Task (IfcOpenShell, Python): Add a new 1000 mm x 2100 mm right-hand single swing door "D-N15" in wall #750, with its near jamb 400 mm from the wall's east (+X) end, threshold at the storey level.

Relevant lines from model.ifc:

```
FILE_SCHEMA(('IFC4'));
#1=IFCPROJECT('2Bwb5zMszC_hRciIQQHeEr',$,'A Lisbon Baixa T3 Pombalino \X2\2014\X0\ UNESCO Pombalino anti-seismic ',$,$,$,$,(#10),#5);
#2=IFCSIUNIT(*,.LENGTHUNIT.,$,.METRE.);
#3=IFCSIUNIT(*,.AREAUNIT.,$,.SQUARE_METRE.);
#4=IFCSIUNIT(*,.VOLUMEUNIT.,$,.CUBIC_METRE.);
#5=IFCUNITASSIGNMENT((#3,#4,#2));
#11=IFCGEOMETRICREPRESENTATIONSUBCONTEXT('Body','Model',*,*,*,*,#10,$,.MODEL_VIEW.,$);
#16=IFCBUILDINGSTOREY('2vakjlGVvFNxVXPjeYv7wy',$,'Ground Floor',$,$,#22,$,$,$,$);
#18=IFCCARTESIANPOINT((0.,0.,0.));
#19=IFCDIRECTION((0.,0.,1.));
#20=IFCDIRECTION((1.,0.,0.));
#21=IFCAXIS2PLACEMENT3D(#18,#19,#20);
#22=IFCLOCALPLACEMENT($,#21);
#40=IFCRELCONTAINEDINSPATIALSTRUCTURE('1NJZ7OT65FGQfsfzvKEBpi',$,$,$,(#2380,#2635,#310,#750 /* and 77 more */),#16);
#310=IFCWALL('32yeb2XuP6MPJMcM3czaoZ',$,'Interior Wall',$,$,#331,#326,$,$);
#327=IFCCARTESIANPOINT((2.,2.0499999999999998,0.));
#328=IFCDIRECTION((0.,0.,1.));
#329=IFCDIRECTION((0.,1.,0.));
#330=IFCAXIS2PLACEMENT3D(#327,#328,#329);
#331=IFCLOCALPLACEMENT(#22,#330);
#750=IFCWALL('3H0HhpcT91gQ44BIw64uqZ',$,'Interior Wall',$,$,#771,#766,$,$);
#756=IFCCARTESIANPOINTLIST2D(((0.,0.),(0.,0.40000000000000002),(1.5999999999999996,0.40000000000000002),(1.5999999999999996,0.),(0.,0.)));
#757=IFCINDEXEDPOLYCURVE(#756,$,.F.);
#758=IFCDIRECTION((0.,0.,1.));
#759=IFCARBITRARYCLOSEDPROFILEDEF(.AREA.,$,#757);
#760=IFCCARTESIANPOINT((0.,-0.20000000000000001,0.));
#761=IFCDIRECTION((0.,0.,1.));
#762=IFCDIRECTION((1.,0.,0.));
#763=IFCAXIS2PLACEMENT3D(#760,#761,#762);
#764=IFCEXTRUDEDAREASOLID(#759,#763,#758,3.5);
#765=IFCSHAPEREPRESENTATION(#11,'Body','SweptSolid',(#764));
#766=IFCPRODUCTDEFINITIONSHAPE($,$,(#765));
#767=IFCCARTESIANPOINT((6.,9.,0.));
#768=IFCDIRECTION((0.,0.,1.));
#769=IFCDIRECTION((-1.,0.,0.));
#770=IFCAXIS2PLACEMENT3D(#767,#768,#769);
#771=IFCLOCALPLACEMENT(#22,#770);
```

```python
import numpy as np
import ifcopenshell
import ifcopenshell.api.feature
import ifcopenshell.api.geometry
import ifcopenshell.api.root
import ifcopenshell.api.spatial
import ifcopenshell.geom
import ifcopenshell.util.element
import ifcopenshell.util.placement
import ifcopenshell.util.representation
import ifcopenshell.util.shape
import ifcopenshell.util.unit

model = ifcopenshell.open("model.ifc")
unit_scale = ifcopenshell.util.unit.calculate_unit_scale(model)
settings = ifcopenshell.geom.settings()


def volume(element):
    """Net volume in cubic metres, openings subtracted."""
    shape = ifcopenshell.geom.create_shape(settings, element)
    return ifcopenshell.util.shape.get_volume(shape.geometry)


wall = model.by_guid("3H0HhpcT91gQ44BIw64uqZ")
storey = ifcopenshell.util.element.get_container(wall, ifc_class="IfcBuildingStorey")
context = ifcopenshell.util.representation.get_context(model, "Model", "Body", "MODEL_VIEW")
before = volume(wall)

width, height, from_end, sill = 1, 2.1, 0.4, 0.0  # metres

# The wall runs along its own X axis, and the end named is its -X end.
wall_shape = ifcopenshell.geom.create_shape(settings, wall)
x, y, z = ifcopenshell.util.shape.get_vertices(wall_shape.geometry).T
start = x.min() + from_end
face, thickness = float(y.min()), float(y.max() - y.min())
wall_matrix = ifcopenshell.util.placement.get_local_placement(wall.ObjectPlacement)
level = ifcopenshell.util.placement.get_local_placement(storey.ObjectPlacement)[2, 3]


def in_wall(x, y):
    """Placement at x, y metres in the wall's axes, at sill height."""
    matrix = wall_matrix.copy()
    matrix[:, 3] = wall_matrix @ np.array([x / unit_scale, y / unit_scale, 0.0, 1.0])
    matrix[2, 3] = level + sill / unit_scale
    return matrix


# Opening: a box that overshoots both wall faces by 50 mm.
opening = ifcopenshell.api.root.create_entity(model, ifc_class="IfcOpeningElement", predefined_type="OPENING")
box = ifcopenshell.api.geometry.add_wall_representation(
    model, context=context, length=width, height=height, thickness=thickness + 0.1
)
ifcopenshell.api.geometry.assign_representation(model, product=opening, representation=box)
ifcopenshell.api.geometry.edit_object_placement(model, product=opening, matrix=in_wall(start, face - 0.05), is_si=False)
ifcopenshell.api.feature.add_feature(model, feature=opening, element=wall)

door = ifcopenshell.api.root.create_entity(model, ifc_class="IfcDoor", name="D-N15", predefined_type="DOOR")
door.OverallWidth, door.OverallHeight = width / unit_scale, height / unit_scale
door.OperationType = "SINGLE_SWING_RIGHT"
body = ifcopenshell.api.geometry.add_door_representation(
    model,
    context=context,
    overall_width=door.OverallWidth,
    overall_height=door.OverallHeight,
    operation_type="SINGLE_SWING_RIGHT",
    lining_properties={"LiningDepth": thickness / unit_scale, "ThresholdDepth": thickness / unit_scale},
)
ifcopenshell.api.geometry.assign_representation(model, product=door, representation=body)
ifcopenshell.api.spatial.assign_container(model, products=[door], relating_structure=storey)
ifcopenshell.api.feature.add_filling(model, opening=opening, element=door)

# The lining spans the wall, so the door starts at the wall face.
ifcopenshell.api.geometry.edit_object_placement(model, product=door, matrix=in_wall(start, face), is_si=False)

after = volume(wall)

print(f"wall volume {before:.3f} -> {after:.3f} m3")

model.write("model_edited.ifc")
```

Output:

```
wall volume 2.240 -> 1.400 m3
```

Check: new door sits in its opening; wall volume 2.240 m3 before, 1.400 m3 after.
